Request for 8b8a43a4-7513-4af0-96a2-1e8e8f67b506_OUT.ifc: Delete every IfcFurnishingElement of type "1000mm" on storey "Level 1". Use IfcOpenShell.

First a look at what the model holds.

```python
import ifcopenshell
import ifcopenshell.util.element

model = ifcopenshell.open("8b8a43a4-7513-4af0-96a2-1e8e8f67b506_OUT.ifc")
print(model.schema)
storey = next(s for s in model.by_type("IfcBuildingStorey") if s.Name == "Level 1")
furniture = [e for e in ifcopenshell.util.element.get_decomposition(storey) if e.is_a("IfcFurnishingElement")]
seen = {}
for e in furniture:
    element_type = ifcopenshell.util.element.get_type(e)
    name = element_type.Name if element_type not in (None, e) else None
    seen[name] = seen.get(name, 0) + 1
for name, count in sorted(seen.items(), key=str):
    print(count, "x", name)
```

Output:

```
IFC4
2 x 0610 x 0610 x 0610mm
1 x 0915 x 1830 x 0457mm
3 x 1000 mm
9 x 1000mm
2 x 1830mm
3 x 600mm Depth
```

```python
import ifcopenshell
import ifcopenshell.api.root
import ifcopenshell.util.element

model = ifcopenshell.open("8b8a43a4-7513-4af0-96a2-1e8e8f67b506_OUT.ifc")

storey = next(s for s in model.by_type("IfcBuildingStorey") if s.Name == "Level 1")
furniture = [e for e in ifcopenshell.util.element.get_decomposition(storey) if e.is_a("IfcFurnishingElement")]
targets = [e for e in furniture if (t := ifcopenshell.util.element.get_type(e)) not in (None, e) and t.Name == "1000mm"]

for e in targets:
    ifcopenshell.api.root.remove_product(model, product=e)
print(len(targets), "removed")

model.write("8b8a43a4-7513-4af0-96a2-1e8e8f67b506_OUT_v2.ifc")
```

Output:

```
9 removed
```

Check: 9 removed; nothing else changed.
